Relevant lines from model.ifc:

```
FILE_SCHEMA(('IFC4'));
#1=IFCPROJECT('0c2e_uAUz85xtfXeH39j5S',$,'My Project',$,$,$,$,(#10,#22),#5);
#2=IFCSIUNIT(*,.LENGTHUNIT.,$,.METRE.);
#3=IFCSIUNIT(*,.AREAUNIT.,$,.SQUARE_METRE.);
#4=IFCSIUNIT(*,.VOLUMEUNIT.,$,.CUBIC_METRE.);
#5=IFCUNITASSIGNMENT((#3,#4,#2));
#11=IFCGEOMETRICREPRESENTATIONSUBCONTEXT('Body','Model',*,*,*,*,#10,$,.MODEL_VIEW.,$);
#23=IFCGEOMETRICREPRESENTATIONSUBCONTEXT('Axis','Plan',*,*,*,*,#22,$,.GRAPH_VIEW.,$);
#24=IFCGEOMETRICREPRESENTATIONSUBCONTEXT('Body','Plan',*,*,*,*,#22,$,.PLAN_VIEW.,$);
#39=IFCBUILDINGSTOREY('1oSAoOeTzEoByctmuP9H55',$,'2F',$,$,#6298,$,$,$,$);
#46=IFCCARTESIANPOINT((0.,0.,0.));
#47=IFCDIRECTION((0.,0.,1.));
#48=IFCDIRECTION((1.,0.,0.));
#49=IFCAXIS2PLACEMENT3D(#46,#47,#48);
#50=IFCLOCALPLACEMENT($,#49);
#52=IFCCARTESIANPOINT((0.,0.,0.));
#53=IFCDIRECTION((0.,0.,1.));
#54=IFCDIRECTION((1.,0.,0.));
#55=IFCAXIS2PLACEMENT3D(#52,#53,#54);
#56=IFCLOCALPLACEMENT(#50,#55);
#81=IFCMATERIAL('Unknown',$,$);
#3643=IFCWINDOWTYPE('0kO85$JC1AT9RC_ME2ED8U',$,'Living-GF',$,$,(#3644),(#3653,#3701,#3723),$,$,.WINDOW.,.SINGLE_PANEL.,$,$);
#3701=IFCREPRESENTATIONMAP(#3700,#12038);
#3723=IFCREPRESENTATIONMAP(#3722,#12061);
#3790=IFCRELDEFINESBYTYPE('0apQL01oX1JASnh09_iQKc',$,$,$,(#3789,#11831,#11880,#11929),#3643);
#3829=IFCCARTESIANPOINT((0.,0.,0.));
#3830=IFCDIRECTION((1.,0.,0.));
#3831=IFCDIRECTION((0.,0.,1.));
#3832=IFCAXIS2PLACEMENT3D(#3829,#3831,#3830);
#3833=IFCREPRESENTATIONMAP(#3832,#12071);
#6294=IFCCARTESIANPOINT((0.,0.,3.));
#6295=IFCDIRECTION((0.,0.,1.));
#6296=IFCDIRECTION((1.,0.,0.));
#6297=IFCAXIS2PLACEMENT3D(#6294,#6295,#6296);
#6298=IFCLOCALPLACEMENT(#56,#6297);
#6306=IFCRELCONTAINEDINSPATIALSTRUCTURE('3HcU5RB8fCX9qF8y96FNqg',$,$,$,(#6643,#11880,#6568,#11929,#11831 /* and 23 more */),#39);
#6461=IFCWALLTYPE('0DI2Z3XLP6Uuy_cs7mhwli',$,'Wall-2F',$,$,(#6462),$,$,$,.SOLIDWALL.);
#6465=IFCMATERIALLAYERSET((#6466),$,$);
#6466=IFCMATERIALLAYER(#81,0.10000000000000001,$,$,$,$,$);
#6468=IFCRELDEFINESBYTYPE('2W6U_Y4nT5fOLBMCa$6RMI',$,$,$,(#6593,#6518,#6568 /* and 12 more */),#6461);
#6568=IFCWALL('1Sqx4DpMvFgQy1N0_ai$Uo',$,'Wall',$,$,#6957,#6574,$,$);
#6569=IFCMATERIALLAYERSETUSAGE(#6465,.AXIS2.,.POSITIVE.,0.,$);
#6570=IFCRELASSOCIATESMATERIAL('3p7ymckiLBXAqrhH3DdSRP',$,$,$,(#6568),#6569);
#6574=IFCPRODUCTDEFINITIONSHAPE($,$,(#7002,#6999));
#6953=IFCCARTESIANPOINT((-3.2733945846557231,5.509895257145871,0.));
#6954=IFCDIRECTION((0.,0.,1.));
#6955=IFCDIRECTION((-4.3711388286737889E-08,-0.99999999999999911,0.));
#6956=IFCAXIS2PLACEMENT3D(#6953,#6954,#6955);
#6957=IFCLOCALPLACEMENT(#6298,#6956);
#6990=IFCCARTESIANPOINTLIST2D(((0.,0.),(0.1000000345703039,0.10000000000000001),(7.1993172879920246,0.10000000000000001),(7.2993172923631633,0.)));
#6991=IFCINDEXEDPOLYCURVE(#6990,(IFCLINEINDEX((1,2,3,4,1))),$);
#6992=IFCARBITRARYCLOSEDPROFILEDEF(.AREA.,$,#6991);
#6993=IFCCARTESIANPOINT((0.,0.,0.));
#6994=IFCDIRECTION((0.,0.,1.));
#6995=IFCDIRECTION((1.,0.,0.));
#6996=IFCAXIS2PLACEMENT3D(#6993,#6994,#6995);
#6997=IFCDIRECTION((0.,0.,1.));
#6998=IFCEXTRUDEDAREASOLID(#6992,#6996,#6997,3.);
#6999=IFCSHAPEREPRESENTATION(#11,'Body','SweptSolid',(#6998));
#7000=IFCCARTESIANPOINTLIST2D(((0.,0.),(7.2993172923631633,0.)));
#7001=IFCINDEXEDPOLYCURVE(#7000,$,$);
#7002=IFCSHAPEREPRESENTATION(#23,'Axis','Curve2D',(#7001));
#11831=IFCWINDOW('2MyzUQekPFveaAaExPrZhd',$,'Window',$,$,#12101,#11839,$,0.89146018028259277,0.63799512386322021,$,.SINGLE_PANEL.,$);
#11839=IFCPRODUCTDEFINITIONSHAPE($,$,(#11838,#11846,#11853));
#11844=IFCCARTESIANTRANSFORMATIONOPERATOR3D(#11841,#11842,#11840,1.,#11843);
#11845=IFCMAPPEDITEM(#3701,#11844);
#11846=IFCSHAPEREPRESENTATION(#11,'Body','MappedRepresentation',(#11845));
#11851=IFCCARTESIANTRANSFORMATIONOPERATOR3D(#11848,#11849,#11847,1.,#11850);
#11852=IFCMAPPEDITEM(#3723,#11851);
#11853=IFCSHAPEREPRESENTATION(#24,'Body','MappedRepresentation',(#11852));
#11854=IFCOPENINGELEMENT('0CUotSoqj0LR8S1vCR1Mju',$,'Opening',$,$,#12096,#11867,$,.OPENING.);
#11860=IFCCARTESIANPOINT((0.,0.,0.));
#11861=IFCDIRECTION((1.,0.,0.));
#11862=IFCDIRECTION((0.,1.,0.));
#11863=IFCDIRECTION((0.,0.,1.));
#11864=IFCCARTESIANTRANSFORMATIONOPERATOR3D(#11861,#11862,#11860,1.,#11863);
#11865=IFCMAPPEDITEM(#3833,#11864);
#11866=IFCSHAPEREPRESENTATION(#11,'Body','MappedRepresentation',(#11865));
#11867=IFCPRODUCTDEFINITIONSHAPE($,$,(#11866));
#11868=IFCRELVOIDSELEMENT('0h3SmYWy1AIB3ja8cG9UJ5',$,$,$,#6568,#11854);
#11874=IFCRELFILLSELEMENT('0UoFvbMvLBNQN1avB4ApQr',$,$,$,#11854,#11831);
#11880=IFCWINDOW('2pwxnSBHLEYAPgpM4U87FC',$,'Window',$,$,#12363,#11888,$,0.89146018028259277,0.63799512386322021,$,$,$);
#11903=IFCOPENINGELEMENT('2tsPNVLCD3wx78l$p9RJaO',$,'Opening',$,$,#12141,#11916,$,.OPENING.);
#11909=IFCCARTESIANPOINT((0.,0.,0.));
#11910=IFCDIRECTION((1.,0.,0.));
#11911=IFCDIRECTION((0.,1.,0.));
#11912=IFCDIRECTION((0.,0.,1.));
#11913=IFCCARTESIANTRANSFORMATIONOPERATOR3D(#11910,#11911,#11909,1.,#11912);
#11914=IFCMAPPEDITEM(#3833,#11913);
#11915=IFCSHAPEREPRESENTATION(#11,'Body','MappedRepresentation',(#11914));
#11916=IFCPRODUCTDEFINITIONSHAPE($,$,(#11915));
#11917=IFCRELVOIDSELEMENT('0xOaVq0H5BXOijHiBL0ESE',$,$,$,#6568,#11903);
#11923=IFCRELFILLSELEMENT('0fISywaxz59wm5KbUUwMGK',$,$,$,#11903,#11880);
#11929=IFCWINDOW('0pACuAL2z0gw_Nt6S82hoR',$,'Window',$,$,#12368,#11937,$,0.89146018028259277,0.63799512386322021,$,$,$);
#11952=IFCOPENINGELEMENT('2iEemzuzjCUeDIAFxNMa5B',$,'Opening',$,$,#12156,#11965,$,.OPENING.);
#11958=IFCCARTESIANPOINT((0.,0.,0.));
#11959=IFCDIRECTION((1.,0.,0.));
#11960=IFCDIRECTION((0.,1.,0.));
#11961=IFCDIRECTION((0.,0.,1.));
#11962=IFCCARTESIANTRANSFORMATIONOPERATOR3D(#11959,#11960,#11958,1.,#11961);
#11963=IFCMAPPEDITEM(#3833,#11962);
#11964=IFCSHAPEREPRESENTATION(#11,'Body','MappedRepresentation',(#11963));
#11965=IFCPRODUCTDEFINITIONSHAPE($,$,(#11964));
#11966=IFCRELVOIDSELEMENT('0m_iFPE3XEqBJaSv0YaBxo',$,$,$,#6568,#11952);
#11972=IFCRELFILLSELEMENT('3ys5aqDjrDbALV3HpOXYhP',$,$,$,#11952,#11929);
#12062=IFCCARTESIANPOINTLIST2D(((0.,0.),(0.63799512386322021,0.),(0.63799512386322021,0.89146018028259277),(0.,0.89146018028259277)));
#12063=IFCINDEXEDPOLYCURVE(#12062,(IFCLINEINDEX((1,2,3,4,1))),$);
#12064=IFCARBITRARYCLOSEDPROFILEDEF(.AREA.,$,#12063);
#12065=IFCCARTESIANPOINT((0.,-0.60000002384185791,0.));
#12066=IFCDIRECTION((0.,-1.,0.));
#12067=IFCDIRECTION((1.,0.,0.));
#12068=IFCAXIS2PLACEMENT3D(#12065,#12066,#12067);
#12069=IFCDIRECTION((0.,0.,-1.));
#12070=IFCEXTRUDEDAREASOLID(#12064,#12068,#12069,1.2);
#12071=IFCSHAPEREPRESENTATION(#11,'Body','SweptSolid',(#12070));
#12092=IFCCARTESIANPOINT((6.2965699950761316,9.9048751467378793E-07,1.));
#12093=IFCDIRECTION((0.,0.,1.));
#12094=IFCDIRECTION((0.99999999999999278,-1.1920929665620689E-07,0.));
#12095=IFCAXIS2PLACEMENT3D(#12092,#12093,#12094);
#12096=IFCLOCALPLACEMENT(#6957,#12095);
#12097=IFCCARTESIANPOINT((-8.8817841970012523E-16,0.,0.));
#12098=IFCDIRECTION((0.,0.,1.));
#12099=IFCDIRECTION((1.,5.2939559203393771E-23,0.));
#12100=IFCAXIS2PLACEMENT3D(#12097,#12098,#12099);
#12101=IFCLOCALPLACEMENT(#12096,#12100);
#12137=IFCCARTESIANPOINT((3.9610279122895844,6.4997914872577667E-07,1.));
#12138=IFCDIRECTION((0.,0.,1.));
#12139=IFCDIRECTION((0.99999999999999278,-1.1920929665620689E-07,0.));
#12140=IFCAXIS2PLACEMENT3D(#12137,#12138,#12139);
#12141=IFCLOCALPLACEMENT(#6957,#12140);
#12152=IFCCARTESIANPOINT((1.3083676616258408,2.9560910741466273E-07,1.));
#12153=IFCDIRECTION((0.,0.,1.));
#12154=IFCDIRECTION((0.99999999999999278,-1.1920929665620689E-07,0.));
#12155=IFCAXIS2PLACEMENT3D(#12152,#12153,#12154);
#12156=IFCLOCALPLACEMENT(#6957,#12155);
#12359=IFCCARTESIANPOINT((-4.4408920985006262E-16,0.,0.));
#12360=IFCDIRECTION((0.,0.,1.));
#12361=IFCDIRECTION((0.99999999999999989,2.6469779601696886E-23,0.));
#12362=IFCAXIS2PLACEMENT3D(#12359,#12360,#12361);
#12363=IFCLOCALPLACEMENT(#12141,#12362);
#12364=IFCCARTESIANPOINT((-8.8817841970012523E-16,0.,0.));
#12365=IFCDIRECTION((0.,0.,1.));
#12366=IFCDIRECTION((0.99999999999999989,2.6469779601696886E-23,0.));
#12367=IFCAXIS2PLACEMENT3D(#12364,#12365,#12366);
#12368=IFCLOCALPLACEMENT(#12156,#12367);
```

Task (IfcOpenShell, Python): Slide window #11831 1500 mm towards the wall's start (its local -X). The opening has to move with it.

```python
import ifcopenshell
import ifcopenshell.api.geometry
import ifcopenshell.util.placement
import ifcopenshell.util.unit

model = ifcopenshell.open("model.ifc")
unit_scale = ifcopenshell.util.unit.calculate_unit_scale(model)

window = model.by_guid("2MyzUQekPFveaAaExPrZhd")
opening = window.FillsVoids[0].RelatingOpeningElement
wall = opening.VoidsElements[0].RelatingBuildingElement

wall_matrix = ifcopenshell.util.placement.get_local_placement(wall.ObjectPlacement)
shift = wall_matrix[:3, 0] * -1.5 / unit_scale
before = ifcopenshell.util.placement.get_local_placement(window.ObjectPlacement)[:3, 3].copy()

# The window is placed relative to its opening, so it follows when the opening moves.
matrix = ifcopenshell.util.placement.get_local_placement(opening.ObjectPlacement)
matrix[:3, 3] += shift
ifcopenshell.api.geometry.edit_object_placement(
    model, product=opening, matrix=matrix, is_si=False, should_transform_children=True
)

after = ifcopenshell.util.placement.get_local_placement(window.ObjectPlacement)[:3, 3]
print("window moved by", (after - before).round(3) + 0.0)

model.write("model_v2.ifc")
```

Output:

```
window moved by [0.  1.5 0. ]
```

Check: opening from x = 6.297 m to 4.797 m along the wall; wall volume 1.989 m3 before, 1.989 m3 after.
